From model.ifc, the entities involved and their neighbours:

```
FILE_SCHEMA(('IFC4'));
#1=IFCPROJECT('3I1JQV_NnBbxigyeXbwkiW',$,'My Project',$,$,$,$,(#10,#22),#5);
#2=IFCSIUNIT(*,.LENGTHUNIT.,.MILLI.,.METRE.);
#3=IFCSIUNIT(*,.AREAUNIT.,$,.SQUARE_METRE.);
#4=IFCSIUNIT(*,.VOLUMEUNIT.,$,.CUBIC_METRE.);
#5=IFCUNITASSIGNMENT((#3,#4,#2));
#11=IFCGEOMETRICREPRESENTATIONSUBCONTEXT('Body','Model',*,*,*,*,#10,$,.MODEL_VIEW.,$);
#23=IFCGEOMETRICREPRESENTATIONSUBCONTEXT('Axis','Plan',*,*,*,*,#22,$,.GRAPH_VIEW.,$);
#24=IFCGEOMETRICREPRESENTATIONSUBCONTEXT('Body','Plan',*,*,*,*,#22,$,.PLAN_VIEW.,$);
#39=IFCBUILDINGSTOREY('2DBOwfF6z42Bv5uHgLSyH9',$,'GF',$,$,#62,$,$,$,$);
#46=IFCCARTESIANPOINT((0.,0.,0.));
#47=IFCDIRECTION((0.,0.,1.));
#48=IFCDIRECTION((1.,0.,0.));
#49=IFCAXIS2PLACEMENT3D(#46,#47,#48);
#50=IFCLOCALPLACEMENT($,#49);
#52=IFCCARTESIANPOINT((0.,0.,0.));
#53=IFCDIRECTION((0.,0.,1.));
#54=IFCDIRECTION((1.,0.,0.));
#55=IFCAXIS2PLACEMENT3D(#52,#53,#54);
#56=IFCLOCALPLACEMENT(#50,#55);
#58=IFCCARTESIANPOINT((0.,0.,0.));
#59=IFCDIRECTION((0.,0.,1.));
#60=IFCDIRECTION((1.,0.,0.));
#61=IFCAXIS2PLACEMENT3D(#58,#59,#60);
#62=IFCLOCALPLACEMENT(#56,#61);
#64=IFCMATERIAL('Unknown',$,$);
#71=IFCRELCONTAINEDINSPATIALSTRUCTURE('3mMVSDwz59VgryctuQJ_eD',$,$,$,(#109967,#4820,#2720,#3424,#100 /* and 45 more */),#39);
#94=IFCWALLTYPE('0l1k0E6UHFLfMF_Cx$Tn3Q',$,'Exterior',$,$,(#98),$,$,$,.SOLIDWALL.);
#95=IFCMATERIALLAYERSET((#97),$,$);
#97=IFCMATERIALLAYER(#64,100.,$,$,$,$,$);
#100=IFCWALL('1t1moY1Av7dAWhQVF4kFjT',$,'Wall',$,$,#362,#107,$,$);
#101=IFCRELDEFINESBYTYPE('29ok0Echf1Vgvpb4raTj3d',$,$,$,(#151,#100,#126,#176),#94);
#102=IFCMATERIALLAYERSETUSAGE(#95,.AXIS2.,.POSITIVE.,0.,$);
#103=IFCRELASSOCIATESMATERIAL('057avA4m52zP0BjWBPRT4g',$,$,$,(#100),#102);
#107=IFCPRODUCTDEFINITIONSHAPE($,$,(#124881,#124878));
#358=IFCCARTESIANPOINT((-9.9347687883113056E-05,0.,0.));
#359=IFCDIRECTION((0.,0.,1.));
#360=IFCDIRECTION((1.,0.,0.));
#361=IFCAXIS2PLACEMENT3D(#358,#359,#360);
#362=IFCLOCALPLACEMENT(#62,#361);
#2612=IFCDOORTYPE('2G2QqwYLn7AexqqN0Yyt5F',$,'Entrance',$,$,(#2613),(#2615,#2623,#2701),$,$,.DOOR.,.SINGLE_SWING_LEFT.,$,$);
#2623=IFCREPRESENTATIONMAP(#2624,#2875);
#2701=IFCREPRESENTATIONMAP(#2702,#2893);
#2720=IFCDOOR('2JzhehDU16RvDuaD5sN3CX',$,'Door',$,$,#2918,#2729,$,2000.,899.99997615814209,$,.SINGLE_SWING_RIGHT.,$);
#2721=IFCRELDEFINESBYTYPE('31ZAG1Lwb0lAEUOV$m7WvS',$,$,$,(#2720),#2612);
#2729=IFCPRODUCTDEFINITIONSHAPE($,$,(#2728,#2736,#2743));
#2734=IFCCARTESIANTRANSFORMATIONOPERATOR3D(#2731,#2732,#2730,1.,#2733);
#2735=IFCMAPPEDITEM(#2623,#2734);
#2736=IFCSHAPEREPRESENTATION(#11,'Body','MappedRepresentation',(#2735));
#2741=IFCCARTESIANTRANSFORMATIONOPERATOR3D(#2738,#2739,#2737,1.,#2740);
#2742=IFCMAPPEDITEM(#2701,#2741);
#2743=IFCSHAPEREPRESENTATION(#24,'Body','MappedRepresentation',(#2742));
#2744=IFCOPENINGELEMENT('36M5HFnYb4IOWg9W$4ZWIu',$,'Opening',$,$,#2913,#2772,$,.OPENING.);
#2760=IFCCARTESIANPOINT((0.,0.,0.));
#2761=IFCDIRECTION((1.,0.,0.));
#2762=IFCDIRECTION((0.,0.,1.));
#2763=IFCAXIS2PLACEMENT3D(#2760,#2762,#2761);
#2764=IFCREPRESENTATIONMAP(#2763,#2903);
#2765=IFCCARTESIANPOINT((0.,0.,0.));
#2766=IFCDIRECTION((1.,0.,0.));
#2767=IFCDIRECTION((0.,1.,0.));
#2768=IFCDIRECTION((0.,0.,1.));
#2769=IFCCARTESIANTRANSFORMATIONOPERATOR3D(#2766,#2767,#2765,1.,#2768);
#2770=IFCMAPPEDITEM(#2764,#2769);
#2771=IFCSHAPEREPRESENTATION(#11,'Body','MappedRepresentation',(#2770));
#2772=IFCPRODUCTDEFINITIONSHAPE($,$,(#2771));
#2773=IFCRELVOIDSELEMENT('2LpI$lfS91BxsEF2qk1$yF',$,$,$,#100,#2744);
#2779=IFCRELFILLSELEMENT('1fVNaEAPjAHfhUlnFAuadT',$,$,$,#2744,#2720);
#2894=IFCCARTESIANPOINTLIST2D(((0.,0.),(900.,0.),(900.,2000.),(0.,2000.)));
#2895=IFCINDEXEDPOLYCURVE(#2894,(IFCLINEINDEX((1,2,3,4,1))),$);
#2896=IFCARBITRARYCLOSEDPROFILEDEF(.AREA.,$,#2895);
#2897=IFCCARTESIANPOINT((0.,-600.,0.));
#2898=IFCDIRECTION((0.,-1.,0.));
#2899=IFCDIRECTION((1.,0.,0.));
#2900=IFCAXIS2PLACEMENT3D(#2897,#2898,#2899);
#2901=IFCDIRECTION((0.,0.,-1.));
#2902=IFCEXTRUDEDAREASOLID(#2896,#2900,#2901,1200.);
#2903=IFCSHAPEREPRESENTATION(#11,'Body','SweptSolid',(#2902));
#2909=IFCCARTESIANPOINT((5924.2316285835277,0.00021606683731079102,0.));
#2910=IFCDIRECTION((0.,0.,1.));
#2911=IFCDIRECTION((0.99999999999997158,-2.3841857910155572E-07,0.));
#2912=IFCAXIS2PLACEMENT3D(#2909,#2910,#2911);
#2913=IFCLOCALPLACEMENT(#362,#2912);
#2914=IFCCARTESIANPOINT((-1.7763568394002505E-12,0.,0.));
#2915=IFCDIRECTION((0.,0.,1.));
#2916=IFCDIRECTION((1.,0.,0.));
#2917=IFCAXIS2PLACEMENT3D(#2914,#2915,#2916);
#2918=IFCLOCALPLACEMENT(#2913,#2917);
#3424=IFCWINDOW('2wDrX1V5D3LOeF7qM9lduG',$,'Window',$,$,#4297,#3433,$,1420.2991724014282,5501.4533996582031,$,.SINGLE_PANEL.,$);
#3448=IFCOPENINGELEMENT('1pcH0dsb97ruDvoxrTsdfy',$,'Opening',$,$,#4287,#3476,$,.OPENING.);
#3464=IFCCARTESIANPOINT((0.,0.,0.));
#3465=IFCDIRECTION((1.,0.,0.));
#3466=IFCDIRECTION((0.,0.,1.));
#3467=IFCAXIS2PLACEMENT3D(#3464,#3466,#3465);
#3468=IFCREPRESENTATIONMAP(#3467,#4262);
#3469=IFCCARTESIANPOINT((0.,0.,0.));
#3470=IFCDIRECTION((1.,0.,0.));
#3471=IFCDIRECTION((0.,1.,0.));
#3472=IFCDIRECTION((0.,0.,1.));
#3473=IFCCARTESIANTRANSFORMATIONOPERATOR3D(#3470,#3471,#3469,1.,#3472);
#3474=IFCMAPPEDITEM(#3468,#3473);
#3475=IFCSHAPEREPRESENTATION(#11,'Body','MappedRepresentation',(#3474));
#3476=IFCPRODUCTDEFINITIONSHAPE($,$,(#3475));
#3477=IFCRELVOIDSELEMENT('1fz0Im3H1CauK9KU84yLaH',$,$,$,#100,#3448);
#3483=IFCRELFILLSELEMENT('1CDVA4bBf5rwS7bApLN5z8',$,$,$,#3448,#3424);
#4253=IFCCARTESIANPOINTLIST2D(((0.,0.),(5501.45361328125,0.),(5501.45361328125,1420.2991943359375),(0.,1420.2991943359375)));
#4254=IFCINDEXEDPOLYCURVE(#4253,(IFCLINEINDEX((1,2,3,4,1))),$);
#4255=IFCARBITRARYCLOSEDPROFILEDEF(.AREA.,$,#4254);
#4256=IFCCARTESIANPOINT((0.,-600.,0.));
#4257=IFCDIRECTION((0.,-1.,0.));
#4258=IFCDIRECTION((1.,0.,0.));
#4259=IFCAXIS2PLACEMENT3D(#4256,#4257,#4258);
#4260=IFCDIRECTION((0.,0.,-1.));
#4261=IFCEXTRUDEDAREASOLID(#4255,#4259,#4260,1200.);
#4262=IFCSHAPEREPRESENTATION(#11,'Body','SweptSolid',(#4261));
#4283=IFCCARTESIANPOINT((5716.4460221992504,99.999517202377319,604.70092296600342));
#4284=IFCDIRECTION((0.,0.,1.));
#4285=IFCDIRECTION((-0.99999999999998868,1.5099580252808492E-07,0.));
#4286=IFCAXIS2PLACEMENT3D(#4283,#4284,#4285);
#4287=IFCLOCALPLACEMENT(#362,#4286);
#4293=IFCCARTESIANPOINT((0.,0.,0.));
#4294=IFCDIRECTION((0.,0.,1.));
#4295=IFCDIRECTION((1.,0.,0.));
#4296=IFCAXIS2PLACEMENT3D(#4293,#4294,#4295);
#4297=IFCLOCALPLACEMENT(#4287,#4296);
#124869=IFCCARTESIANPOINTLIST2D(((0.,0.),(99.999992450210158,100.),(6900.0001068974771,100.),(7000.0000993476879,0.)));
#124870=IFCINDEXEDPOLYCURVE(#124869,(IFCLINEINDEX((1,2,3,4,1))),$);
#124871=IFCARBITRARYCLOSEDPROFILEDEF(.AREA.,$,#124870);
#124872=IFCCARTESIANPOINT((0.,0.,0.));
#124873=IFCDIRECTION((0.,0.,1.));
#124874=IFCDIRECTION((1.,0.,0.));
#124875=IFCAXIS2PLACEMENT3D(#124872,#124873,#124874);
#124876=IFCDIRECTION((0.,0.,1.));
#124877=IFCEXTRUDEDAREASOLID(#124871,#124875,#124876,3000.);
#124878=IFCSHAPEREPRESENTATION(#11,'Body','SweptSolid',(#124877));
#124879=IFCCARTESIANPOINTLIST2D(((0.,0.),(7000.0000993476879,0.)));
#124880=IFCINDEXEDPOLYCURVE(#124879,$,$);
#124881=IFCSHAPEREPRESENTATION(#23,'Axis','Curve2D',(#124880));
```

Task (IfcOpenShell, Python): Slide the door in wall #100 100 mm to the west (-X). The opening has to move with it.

```python
import ifcopenshell
import ifcopenshell.api.geometry
import ifcopenshell.util.placement
import ifcopenshell.util.unit

model = ifcopenshell.open("model.ifc")
unit_scale = ifcopenshell.util.unit.calculate_unit_scale(model)

door = model.by_id(2720)
opening = door.FillsVoids[0].RelatingOpeningElement
wall = opening.VoidsElements[0].RelatingBuildingElement

wall_matrix = ifcopenshell.util.placement.get_local_placement(wall.ObjectPlacement)
shift = wall_matrix[:3, 0] * -0.1 / unit_scale
before = ifcopenshell.util.placement.get_local_placement(door.ObjectPlacement)[:3, 3].copy()

# The door is placed relative to its opening, so it follows when the opening moves.
matrix = ifcopenshell.util.placement.get_local_placement(opening.ObjectPlacement)
matrix[:3, 3] += shift
ifcopenshell.api.geometry.edit_object_placement(
    model, product=opening, matrix=matrix, is_si=False, should_transform_children=True
)

after = ifcopenshell.util.placement.get_local_placement(door.ObjectPlacement)[:3, 3]
print("door moved by", (after - before).round(3) + 0.0)

model.write("model_v2.ifc")
```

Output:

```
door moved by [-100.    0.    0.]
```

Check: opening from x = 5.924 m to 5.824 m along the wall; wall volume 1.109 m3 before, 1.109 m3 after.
